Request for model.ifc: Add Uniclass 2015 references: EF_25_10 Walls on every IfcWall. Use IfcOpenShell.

First a look at what the model holds.

```python
import ifcopenshell

model = ifcopenshell.open("model.ifc")
print(model.schema)
print("classifications:", [c.Name for c in model.by_type("IfcClassification")])
for ifc_class in ("IfcDoor", "IfcRoof", "IfcStair", "IfcWall", "IfcWindow"):
    print(ifc_class, len(model.by_type(ifc_class)))
```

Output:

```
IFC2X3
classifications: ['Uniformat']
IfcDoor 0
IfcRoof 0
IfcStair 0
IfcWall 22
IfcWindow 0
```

```python
import ifcopenshell
import ifcopenshell.api.classification

model = ifcopenshell.open("model.ifc")

# IFC2X3 requires Source and Edition and has no link from the project to the system.
system = model.create_entity("IfcClassification", Source="NBS", Edition="2015", Name="Uniclass 2015")

codes = {
    "IfcWall": ("EF_25_10", "Walls"),
}
for ifc_class, (code, name) in codes.items():
    products = model.by_type(ifc_class)
    ifcopenshell.api.classification.add_reference(
        model, products=products, classification=system, identification=code, name=name
    )
    print(code, len(products))

model.write("model_edited.ifc")
```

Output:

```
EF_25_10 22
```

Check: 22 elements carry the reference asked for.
